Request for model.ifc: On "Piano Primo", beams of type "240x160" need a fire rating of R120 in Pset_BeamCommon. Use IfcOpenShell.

First a look at what the model holds.

```python
import ifcopenshell
import ifcopenshell.util.element

model = ifcopenshell.open("model.ifc")
print(model.schema)
storey = next(s for s in model.by_type("IfcBuildingStorey") if s.Name == "Piano Primo")
beams = [e for e in ifcopenshell.util.element.get_decomposition(storey) if e.is_a("IfcBeam")]
seen = {}
for e in beams:
    element_type = ifcopenshell.util.element.get_type(e)
    key = (element_type.Name if element_type != e and element_type else None, ifcopenshell.util.element.get_pset(e, "Pset_BeamCommon", "FireRating"))
    seen[key] = seen.get(key, 0) + 1
for (name, value), count in sorted(seen.items(), key=str):
    print(count, "x", name, "|", value)
```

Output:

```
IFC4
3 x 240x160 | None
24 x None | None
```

```python
import ifcopenshell
import ifcopenshell.api.pset
import ifcopenshell.util.element

model = ifcopenshell.open("model.ifc")

storey = next(s for s in model.by_type("IfcBuildingStorey") if s.Name == "Piano Primo")
beams = [e for e in ifcopenshell.util.element.get_decomposition(storey) if e.is_a("IfcBeam")]

count = 0
for e in beams:
    element_type = ifcopenshell.util.element.get_type(e)
    if element_type in (None, e) or element_type.Name != "240x160":
        continue
    # add_pset returns the element's existing set when there is one.
    pset = ifcopenshell.api.pset.add_pset(model, product=e, name="Pset_BeamCommon")
    ifcopenshell.api.pset.edit_pset(model, pset=pset, properties={"FireRating": "R120"})
    count += 1

print(count, "beams updated")

model.write("model_updated.ifc")
```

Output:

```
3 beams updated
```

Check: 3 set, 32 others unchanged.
